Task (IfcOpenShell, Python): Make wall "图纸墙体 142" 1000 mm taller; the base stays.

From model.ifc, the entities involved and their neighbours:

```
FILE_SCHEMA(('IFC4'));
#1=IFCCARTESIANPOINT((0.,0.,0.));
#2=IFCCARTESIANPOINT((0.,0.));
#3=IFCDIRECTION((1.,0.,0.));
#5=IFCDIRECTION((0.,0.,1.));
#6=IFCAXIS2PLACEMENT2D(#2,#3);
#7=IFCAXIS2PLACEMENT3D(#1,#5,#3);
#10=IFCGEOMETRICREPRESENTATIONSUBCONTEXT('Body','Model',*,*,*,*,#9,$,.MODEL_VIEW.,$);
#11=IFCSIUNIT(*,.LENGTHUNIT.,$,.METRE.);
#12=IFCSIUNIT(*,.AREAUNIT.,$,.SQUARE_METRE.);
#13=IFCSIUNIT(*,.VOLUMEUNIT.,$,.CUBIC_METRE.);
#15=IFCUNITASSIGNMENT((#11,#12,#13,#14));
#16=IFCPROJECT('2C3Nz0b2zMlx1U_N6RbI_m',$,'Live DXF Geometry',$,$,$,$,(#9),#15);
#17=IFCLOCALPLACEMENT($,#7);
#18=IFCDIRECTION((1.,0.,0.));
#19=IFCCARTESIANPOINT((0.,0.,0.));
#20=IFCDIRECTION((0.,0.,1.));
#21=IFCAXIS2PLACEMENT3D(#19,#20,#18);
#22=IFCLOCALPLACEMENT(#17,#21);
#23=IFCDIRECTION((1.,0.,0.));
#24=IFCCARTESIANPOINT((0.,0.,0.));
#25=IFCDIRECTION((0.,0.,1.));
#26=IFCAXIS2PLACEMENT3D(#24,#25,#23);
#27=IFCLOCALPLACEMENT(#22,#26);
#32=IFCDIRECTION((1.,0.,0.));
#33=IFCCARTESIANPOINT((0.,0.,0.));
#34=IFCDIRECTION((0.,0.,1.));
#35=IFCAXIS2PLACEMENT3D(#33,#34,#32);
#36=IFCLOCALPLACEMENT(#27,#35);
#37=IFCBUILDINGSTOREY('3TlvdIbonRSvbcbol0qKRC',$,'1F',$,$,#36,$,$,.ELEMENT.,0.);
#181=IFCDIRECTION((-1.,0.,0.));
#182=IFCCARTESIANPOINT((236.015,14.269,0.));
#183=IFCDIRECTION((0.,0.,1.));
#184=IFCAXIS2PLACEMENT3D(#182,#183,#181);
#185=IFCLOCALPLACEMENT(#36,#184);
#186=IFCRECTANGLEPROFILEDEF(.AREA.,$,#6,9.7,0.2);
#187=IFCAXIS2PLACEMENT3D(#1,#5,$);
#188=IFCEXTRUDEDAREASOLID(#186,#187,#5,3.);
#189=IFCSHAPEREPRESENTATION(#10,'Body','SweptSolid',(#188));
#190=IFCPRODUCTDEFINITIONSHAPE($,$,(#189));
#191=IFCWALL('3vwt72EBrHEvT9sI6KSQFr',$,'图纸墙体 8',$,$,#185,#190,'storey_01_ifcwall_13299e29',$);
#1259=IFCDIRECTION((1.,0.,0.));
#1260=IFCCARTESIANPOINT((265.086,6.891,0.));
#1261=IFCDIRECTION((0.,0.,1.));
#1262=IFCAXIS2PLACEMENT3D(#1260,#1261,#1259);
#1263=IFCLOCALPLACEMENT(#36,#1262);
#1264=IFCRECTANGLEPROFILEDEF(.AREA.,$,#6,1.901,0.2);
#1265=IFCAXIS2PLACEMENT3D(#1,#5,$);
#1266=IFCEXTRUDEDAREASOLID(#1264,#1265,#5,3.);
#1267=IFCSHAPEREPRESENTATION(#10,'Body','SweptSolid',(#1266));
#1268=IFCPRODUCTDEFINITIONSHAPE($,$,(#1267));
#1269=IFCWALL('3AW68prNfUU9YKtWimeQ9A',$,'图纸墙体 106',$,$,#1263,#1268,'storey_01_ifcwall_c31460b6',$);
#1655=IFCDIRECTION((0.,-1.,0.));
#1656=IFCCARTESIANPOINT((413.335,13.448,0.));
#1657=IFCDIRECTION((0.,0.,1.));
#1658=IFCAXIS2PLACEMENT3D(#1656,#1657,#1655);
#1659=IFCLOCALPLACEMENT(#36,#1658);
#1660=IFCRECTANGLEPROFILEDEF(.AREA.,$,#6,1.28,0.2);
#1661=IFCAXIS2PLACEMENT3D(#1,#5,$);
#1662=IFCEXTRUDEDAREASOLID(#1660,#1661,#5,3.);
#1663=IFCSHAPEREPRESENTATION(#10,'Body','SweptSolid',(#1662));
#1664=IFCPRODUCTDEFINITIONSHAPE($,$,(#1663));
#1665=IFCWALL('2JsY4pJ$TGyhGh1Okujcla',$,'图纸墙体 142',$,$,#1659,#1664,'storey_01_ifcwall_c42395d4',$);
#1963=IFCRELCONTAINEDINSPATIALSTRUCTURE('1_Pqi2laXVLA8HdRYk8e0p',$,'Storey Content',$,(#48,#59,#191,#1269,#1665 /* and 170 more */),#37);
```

```python
import ifcopenshell
import ifcopenshell.geom
import ifcopenshell.util.representation
import ifcopenshell.util.shape
import ifcopenshell.util.unit

model = ifcopenshell.open("model.ifc")
unit_scale = ifcopenshell.util.unit.calculate_unit_scale(model)
settings = ifcopenshell.geom.settings()


def volume(element):
    """Net volume in cubic metres, openings subtracted."""
    shape = ifcopenshell.geom.create_shape(settings, element)
    return ifcopenshell.util.shape.get_volume(shape.geometry)


wall = model.by_guid("2JsY4pJ$TGyhGh1Okujcla")
before = volume(wall)

body = ifcopenshell.util.representation.get_representation(wall, "Model", "Body")
solid = body.Items[0]
old_height = solid.Depth
solid.Depth += 1 / unit_scale
after = volume(wall)

print(f"height {old_height:g} -> {solid.Depth:g}, volume {before:.3f} -> {after:.3f} m3")

model.write("model-out.ifc")
```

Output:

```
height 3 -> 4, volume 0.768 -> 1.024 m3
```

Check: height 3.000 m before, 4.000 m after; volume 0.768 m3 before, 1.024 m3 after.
